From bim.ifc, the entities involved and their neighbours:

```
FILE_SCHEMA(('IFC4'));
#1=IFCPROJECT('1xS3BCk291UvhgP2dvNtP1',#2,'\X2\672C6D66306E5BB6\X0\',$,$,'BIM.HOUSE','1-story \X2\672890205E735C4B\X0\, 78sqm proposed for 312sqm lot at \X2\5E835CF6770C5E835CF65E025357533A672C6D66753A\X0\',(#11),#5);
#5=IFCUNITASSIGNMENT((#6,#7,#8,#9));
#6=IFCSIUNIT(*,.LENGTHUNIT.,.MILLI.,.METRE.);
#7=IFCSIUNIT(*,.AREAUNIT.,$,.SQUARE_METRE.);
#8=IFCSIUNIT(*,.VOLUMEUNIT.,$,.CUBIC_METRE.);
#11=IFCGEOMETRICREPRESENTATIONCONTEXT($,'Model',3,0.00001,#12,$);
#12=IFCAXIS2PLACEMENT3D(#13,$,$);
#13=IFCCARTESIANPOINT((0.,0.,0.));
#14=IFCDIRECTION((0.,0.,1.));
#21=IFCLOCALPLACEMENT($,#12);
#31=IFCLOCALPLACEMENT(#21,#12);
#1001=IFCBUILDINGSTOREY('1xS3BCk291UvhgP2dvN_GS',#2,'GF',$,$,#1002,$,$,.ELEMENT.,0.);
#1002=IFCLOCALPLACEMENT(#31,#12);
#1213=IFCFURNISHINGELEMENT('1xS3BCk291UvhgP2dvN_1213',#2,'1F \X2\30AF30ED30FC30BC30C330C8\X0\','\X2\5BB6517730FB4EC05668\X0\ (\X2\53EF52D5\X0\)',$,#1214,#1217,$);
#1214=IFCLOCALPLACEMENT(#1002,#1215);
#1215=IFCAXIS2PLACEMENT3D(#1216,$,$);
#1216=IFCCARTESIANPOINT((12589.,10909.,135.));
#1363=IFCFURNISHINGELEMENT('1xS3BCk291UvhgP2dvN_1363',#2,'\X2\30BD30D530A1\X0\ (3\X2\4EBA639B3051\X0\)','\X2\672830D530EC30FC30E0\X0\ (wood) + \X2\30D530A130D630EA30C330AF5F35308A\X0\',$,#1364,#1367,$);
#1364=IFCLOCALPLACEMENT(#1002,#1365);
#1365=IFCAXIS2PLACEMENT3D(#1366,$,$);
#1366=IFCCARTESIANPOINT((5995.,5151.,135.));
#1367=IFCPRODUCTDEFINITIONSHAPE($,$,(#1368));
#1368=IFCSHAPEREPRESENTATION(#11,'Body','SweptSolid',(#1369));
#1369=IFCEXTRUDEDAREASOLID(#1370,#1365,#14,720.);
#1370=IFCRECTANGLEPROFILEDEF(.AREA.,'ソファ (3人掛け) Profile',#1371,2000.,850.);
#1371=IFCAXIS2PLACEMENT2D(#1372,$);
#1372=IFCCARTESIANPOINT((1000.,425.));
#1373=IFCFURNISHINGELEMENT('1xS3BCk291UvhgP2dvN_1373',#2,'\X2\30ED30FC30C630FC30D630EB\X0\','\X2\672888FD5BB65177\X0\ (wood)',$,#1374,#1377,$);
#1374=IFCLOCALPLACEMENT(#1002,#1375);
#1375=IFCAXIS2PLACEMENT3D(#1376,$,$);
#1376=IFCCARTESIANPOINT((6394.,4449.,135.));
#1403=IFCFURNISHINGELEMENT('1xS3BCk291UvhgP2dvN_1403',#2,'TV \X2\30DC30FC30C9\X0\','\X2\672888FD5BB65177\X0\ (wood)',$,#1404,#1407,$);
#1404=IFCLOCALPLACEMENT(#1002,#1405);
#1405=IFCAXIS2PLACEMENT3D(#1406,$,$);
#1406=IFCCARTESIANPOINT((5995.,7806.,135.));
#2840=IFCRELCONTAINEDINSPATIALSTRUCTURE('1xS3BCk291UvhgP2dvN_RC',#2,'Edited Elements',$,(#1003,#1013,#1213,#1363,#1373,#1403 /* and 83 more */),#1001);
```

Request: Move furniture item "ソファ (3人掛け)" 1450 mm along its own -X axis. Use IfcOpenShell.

```python
import ifcopenshell
import ifcopenshell.api.geometry
import ifcopenshell.util.placement

model = ifcopenshell.open("bim.ifc")

item = model.by_id(1363)
matrix = ifcopenshell.util.placement.get_local_placement(item.ObjectPlacement)
matrix[:3, 3] -= matrix[:3, 0] * 1450.0
ifcopenshell.api.geometry.edit_object_placement(model, product=item, matrix=matrix, is_si=False)

print(ifcopenshell.util.placement.get_local_placement(item.ObjectPlacement).round(3) + 0.0)

model.write("bim_edited.ifc")
```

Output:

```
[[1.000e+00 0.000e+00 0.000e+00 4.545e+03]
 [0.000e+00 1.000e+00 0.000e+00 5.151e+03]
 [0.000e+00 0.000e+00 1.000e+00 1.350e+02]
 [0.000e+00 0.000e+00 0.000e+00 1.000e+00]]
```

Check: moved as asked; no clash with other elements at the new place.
